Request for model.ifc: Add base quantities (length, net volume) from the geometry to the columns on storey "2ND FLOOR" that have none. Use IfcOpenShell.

First a look at what the model holds.

```python
import ifcopenshell
import ifcopenshell.util.element
import ifcopenshell.util.unit

model = ifcopenshell.open("model.ifc")
print(model.schema)
for unit_type in ("LENGTHUNIT", "AREAUNIT", "VOLUMEUNIT"):
    print(unit_type, ifcopenshell.util.unit.calculate_unit_scale(model, unit_type))
storey = next(s for s in model.by_type("IfcBuildingStorey") if s.Name == "2ND FLOOR")
columns = [e for e in ifcopenshell.util.element.get_decomposition(storey) if e.is_a("IfcColumn")]
for e in sorted(columns, key=lambda e: e.id()):
    print(e.id(), e.is_a(), e.Name, list(ifcopenshell.util.element.get_psets(e, qtos_only=True)), sep=" | ")
```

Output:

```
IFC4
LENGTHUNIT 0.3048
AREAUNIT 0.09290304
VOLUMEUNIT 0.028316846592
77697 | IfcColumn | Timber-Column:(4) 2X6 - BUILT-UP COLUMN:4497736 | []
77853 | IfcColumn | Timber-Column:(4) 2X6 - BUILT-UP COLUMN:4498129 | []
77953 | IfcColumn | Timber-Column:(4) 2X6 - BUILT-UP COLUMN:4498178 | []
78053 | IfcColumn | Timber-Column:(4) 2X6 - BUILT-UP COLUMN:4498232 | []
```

```python
import ifcopenshell
import ifcopenshell.api.pset
import ifcopenshell.geom
import ifcopenshell.util.element
import ifcopenshell.util.shape
import ifcopenshell.util.unit

model = ifcopenshell.open("model.ifc")
unit_scale = ifcopenshell.util.unit.calculate_unit_scale(model)
volume_scale = ifcopenshell.util.unit.calculate_unit_scale(model, "VOLUMEUNIT")
settings = ifcopenshell.geom.settings()

storey = next(s for s in model.by_type("IfcBuildingStorey") if s.Name == "2ND FLOOR")
columns = [e for e in ifcopenshell.util.element.get_decomposition(storey) if e.is_a("IfcColumn")]

for e in sorted(columns, key=lambda e: e.id()):
    if ifcopenshell.util.element.get_psets(e, qtos_only=True, should_inherit=False):
        continue
    # Geometry comes back in metres, in the element's own axes.
    shape = ifcopenshell.geom.create_shape(settings, e)
    values = {
        "Length": ifcopenshell.util.shape.get_z(shape.geometry) / unit_scale,
        "NetVolume": ifcopenshell.util.shape.get_volume(shape.geometry) / volume_scale,
    }
    qto = ifcopenshell.api.pset.add_qto(model, product=e, name="Qto_ColumnBaseQuantities")
    ifcopenshell.api.pset.edit_qto(model, qto=qto, properties=values)
    print(e.id(), {k: round(v, 3) for k, v in values.items()})

model.write("model-out.ifc")
```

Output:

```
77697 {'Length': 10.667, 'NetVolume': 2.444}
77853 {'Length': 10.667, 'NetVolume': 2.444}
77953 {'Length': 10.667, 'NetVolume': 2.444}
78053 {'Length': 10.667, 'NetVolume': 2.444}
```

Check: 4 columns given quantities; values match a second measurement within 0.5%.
